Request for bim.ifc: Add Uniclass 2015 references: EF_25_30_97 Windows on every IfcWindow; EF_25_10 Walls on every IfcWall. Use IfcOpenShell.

First a look at what the model holds.

```python
import ifcopenshell

model = ifcopenshell.open("bim.ifc")
print(model.schema)
print("classifications:", [c.Name for c in model.by_type("IfcClassification")])
for ifc_class in ("IfcDoor", "IfcRoof", "IfcStair", "IfcWall", "IfcWindow"):
    print(ifc_class, len(model.by_type(ifc_class)))
```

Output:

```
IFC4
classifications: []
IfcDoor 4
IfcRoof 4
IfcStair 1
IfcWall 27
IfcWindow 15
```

```python
import ifcopenshell
import ifcopenshell.api.classification

model = ifcopenshell.open("bim.ifc")

system = ifcopenshell.api.classification.add_classification(model, classification="Uniclass 2015")

codes = {
    "IfcWindow": ("EF_25_30_97", "Windows"),
    "IfcWall": ("EF_25_10", "Walls"),
}
for ifc_class, (code, name) in codes.items():
    products = model.by_type(ifc_class)
    ifcopenshell.api.classification.add_reference(
        model, products=products, classification=system, identification=code, name=name
    )
    print(code, len(products))

model.write("bim_rev.ifc")
```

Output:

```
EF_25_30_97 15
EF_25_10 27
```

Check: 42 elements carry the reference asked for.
